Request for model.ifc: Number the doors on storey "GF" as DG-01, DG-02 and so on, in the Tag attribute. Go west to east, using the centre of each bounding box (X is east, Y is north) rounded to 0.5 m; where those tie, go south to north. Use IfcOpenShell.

First a look at what the model holds.

```python
import ifcopenshell
import ifcopenshell.util.element
import ifcopenshell.util.placement

model = ifcopenshell.open("model.ifc")
print(model.schema)
storey = next(s for s in model.by_type("IfcBuildingStorey") if s.Name == "GF")
doors = [e for e in ifcopenshell.util.element.get_decomposition(storey) if e.is_a("IfcDoor")]
for e in sorted(doors, key=lambda e: e.id()):
    origin = ifcopenshell.util.placement.get_local_placement(e.ObjectPlacement)[:3, 3]
    print(e.id(), e.Tag, e.Name, origin.round(2) + 0.0, sep=" | ")
```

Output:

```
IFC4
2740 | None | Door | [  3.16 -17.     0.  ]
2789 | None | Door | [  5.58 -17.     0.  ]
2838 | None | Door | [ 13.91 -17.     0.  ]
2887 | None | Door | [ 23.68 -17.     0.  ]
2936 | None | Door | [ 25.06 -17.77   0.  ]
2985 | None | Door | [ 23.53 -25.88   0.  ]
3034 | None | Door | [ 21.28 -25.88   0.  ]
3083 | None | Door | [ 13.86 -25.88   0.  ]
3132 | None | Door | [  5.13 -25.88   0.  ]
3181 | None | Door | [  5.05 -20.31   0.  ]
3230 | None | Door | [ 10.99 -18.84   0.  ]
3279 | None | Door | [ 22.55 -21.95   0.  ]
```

```python
import ifcopenshell
import ifcopenshell.geom
import ifcopenshell.util.element
import ifcopenshell.util.shape

model = ifcopenshell.open("model.ifc")
settings = ifcopenshell.geom.settings()
settings.set("use-world-coords", True)


def centre(element):
    shape = ifcopenshell.geom.create_shape(settings, element)
    return ifcopenshell.util.shape.get_bbox_centroid(shape.geometry)


storey = next(s for s in model.by_type("IfcBuildingStorey") if s.Name == "GF")
doors = [e for e in ifcopenshell.util.element.get_decomposition(storey) if e.is_a("IfcDoor")]

# Insertion points can sit at a corner or the storey origin, so sort by the geometry (in metres).
centres = {e: centre(e) for e in doors}
doors.sort(key=lambda e: (round(centres[e][0] / 0.5), centres[e][1]))

for i, e in enumerate(doors, start=1):
    number = f"DG-{i:02d}"
    e.Tag = number
    print(e.id(), number)

model.write("model-out.ifc")
```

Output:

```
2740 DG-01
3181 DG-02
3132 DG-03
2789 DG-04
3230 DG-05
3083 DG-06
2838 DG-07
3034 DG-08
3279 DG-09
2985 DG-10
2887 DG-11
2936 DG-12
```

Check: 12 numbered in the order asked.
